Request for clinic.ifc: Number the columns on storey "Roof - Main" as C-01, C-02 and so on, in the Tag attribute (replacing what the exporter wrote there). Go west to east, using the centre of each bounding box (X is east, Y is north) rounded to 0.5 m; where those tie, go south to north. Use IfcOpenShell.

First a look at what the model holds.

```python
import ifcopenshell
import ifcopenshell.util.element
import ifcopenshell.util.placement

model = ifcopenshell.open("clinic.ifc")
print(model.schema)
storey = next(s for s in model.by_type("IfcBuildingStorey") if s.Name == "Roof - Main")
columns = [e for e in ifcopenshell.util.element.get_decomposition(storey) if e.is_a("IfcColumn")]
for e in sorted(columns, key=lambda e: e.id()):
    origin = ifcopenshell.util.placement.get_local_placement(e.ObjectPlacement)[:3, 3]
    print(e.id(), e.Tag, e.Name, origin.round(2) + 0.0, sep=" | ")
```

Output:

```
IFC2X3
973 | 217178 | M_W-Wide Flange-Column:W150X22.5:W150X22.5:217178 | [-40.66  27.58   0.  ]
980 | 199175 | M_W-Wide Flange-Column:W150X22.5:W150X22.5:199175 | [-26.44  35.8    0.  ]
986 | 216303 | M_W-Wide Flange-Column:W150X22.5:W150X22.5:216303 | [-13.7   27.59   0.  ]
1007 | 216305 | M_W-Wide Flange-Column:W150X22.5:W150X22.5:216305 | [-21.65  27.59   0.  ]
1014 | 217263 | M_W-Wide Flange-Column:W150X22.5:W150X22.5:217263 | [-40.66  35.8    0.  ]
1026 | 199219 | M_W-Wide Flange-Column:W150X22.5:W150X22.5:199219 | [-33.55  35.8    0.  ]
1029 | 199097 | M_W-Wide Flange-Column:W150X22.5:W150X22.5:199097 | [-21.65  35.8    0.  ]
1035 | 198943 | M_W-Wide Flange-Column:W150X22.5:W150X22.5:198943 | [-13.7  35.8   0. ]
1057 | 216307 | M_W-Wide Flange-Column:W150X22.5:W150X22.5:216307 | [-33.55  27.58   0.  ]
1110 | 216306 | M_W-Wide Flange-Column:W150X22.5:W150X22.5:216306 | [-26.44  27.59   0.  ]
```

```python
import ifcopenshell
import ifcopenshell.geom
import ifcopenshell.util.element
import ifcopenshell.util.shape

model = ifcopenshell.open("clinic.ifc")
settings = ifcopenshell.geom.settings()
settings.set("use-world-coords", True)


def centre(element):
    shape = ifcopenshell.geom.create_shape(settings, element)
    return ifcopenshell.util.shape.get_bbox_centroid(shape.geometry)


storey = next(s for s in model.by_type("IfcBuildingStorey") if s.Name == "Roof - Main")
columns = [e for e in ifcopenshell.util.element.get_decomposition(storey) if e.is_a("IfcColumn")]

# Insertion points can sit at a corner or the storey origin, so sort by the geometry (in metres).
centres = {e: centre(e) for e in columns}
columns.sort(key=lambda e: (round(centres[e][0] / 0.5), centres[e][1]))

for i, e in enumerate(columns, start=1):
    number = f"C-{i:02d}"
    e.Tag = number
    print(e.id(), number)

model.write("clinic_v2.ifc")
```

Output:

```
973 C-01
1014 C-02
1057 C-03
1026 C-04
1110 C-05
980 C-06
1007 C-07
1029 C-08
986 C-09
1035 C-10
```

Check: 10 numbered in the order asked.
